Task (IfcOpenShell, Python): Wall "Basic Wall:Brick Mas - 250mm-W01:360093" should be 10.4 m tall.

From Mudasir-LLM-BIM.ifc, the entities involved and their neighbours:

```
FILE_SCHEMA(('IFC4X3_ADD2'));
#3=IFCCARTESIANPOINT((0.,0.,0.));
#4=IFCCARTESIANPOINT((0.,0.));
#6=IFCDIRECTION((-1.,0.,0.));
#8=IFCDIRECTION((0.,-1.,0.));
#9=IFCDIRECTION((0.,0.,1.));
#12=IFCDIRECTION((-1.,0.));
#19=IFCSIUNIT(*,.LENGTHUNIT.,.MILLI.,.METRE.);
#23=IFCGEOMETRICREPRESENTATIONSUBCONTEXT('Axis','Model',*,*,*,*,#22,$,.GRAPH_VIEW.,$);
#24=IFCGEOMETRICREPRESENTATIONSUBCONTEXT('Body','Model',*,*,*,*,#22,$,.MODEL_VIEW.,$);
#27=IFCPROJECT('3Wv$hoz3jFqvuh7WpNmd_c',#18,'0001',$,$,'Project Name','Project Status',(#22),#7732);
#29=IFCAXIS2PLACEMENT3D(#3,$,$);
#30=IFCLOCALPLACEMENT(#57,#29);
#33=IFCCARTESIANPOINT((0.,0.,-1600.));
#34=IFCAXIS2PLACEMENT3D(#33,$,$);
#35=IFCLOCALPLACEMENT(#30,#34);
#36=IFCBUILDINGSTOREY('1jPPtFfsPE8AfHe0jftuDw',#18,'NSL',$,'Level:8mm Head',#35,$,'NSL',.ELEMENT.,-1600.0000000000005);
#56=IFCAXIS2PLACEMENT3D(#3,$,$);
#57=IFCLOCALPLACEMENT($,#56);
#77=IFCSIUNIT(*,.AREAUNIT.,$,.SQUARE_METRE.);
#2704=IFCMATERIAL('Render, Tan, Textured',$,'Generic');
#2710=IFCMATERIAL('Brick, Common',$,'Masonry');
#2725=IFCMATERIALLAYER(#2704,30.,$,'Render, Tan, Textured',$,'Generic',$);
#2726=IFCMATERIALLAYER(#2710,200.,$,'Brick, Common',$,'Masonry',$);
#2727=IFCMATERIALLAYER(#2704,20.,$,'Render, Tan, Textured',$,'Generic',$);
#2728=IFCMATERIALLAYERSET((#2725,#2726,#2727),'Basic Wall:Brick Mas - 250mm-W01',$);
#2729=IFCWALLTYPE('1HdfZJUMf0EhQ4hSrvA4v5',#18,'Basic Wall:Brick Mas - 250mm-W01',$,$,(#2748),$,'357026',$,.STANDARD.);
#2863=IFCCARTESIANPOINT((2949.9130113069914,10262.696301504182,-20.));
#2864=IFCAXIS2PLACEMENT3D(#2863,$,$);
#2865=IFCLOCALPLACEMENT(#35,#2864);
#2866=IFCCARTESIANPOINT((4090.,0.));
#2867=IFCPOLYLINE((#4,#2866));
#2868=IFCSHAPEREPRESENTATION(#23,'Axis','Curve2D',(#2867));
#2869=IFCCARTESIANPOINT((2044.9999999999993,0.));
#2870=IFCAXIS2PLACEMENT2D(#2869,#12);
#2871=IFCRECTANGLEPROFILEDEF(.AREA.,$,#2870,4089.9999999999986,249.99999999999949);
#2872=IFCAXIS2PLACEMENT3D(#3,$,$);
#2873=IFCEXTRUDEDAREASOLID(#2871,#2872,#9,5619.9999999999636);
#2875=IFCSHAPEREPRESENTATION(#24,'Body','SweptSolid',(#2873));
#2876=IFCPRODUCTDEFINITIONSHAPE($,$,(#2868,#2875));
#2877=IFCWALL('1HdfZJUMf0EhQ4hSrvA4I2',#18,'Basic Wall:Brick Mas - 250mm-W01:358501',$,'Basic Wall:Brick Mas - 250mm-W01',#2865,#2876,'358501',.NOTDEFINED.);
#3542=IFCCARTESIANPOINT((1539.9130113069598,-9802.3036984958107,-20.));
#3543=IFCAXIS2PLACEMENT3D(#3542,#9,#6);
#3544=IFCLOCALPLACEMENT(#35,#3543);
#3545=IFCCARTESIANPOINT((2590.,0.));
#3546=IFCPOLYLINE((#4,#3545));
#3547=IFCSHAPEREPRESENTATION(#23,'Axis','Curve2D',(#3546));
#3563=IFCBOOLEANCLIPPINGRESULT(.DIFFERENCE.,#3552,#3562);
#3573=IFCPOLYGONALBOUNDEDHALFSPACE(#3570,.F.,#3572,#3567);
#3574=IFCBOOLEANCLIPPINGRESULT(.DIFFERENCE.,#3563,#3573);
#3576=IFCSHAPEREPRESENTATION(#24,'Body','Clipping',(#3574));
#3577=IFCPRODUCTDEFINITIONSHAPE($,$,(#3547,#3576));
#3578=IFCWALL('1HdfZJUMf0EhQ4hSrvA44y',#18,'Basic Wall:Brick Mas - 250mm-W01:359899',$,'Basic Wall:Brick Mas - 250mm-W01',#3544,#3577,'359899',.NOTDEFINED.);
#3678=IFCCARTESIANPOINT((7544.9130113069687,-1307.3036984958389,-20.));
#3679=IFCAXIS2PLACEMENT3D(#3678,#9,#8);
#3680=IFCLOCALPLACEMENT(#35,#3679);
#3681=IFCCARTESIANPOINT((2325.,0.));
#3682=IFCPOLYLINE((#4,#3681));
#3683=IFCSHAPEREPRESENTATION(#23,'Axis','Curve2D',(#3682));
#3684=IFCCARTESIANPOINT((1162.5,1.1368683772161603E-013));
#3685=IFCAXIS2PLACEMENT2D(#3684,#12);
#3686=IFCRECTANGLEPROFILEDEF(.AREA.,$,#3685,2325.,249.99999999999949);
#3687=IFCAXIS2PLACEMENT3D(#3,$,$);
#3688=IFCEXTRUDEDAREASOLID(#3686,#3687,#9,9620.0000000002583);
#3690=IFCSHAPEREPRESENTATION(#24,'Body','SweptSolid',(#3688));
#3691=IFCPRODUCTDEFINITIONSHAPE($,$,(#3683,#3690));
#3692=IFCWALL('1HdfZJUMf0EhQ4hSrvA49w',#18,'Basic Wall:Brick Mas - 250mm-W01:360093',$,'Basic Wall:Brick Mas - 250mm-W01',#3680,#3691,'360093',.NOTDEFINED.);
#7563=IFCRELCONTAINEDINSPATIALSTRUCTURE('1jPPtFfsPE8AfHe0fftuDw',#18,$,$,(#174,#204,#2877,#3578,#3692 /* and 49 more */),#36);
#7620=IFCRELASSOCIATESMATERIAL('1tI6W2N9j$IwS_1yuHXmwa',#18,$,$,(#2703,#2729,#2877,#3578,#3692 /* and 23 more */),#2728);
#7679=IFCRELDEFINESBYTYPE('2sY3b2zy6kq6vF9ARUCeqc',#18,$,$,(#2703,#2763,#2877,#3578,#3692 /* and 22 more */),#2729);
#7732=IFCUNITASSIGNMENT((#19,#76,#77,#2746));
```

```python
import ifcopenshell
import ifcopenshell.geom
import ifcopenshell.util.representation
import ifcopenshell.util.shape

model = ifcopenshell.open("Mudasir-LLM-BIM.ifc")
settings = ifcopenshell.geom.settings()


def volume(element):
    """Net volume in cubic metres, openings subtracted."""
    shape = ifcopenshell.geom.create_shape(settings, element)
    return ifcopenshell.util.shape.get_volume(shape.geometry)


wall = model.by_guid("1HdfZJUMf0EhQ4hSrvA49w")
before = volume(wall)

body = ifcopenshell.util.representation.get_representation(wall, "Model", "Body")
solid = body.Items[0]
old_height = solid.Depth
solid.Depth = 10400.0
after = volume(wall)

print(f"height {old_height:g} -> {solid.Depth:g}, volume {before:.3f} -> {after:.3f} m3")

model.write("Mudasir-LLM-BIM_v2.ifc")
```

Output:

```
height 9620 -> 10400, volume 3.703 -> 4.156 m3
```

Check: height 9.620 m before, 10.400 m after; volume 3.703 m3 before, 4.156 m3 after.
